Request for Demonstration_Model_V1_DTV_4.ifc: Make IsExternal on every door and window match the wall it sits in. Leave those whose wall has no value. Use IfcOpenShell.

First a look at what the model holds.

```python
import ifcopenshell
import ifcopenshell.util.element

model = ifcopenshell.open("Demonstration_Model_V1_DTV_4.ifc")
print(model.schema)
seen = {}
for e in model.by_type("IfcDoor") + model.by_type("IfcWindow"):
    if not e.FillsVoids:
        continue
    host = e.FillsVoids[0].RelatingOpeningElement.VoidsElements[0].RelatingBuildingElement
    own = ifcopenshell.util.element.get_pset(e, f"Pset_{e.is_a()[3:].removesuffix('StandardCase')}Common", "IsExternal")
    wall = ifcopenshell.util.element.get_pset(host, "Pset_WallCommon", "IsExternal")
    seen[e.is_a(), own, wall] = seen.get((e.is_a(), own, wall), 0) + 1
for (cls, own, wall), count in sorted(seen.items(), key=str):
    print(count, cls, "IsExternal:", own, "| host wall:", wall)
```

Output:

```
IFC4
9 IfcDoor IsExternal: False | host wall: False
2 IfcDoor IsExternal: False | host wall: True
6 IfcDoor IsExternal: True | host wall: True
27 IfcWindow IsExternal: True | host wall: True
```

```python
import ifcopenshell
import ifcopenshell.api.pset
import ifcopenshell.util.element

model = ifcopenshell.open("Demonstration_Model_V1_DTV_4.ifc")

count = 0
for ifc_class, pset_name in (("IfcDoor", "Pset_DoorCommon"), ("IfcWindow", "Pset_WindowCommon")):
    for e in model.by_type(ifc_class):
        if not e.FillsVoids:
            continue
        host = e.FillsVoids[0].RelatingOpeningElement.VoidsElements[0].RelatingBuildingElement
        external = ifcopenshell.util.element.get_pset(host, "Pset_WallCommon", "IsExternal")
        if external is None or ifcopenshell.util.element.get_pset(e, pset_name, "IsExternal") == external:
            continue
        pset = ifcopenshell.api.pset.add_pset(model, product=e, name=pset_name)
        ifcopenshell.api.pset.edit_pset(model, pset=pset, properties={"IsExternal": external})
        count += 1

print(count, "updated")

model.write("Demonstration_Model_V1_DTV_4_updated.ifc")
```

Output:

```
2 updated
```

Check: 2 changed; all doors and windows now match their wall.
